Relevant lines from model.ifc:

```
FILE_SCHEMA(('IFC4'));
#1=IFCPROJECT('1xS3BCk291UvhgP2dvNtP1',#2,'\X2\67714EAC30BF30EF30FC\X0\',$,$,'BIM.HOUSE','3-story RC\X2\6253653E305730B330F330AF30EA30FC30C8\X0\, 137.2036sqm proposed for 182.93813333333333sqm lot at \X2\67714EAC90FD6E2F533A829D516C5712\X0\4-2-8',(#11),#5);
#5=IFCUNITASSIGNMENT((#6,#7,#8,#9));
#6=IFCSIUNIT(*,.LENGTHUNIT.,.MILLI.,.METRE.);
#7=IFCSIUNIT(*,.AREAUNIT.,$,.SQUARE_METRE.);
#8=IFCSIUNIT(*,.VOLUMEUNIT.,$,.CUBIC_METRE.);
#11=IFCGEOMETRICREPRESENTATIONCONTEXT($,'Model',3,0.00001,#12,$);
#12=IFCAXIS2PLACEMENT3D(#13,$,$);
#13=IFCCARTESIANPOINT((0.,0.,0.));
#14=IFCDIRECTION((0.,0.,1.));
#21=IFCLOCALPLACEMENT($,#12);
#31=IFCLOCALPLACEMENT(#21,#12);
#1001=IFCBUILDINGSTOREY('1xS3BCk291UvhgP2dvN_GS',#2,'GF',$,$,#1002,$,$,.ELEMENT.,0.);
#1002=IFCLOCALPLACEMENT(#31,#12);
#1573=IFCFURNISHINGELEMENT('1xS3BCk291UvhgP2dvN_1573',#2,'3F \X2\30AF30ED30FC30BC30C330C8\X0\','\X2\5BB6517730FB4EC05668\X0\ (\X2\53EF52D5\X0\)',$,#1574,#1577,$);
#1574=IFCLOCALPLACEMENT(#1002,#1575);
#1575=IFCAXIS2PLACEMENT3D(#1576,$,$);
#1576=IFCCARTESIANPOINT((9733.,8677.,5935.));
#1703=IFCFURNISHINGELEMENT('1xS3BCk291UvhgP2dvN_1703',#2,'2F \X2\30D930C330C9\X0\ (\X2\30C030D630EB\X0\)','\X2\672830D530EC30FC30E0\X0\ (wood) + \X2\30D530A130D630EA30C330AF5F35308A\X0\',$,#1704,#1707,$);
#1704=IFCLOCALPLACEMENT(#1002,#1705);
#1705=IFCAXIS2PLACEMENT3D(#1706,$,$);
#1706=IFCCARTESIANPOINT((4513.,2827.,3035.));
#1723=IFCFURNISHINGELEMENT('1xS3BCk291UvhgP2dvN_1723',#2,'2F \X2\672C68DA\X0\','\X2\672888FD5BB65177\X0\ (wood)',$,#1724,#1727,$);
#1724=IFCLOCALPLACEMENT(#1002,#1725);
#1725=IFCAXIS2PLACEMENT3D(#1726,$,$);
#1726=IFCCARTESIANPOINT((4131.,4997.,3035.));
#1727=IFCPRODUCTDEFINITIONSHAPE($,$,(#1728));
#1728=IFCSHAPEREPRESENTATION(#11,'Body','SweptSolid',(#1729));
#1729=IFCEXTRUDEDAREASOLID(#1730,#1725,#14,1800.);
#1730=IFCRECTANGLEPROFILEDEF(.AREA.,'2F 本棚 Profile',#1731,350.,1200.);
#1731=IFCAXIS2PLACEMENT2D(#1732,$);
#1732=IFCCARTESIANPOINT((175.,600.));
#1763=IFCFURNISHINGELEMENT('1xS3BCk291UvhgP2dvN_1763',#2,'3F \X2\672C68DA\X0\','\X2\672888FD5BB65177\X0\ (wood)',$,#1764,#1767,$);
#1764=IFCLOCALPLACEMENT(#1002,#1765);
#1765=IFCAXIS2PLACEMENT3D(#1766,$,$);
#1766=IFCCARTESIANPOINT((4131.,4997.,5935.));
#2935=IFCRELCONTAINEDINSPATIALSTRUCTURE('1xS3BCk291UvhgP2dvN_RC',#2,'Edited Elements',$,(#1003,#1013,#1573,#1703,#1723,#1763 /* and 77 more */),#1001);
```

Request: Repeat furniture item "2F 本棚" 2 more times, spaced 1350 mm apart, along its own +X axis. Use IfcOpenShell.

```python
import ifcopenshell
import ifcopenshell.api.geometry
import ifcopenshell.api.root
import ifcopenshell.util.element
import ifcopenshell.util.placement
import ifcopenshell.util.unit

model = ifcopenshell.open("model.ifc")
unit_scale = ifcopenshell.util.unit.calculate_unit_scale(model)


def reuse_history(source, copy):
    """copy_class also copies each property set's owner history, people and application; keep the originals."""
    for rel in copy.IsDefinedBy:
        if rel.is_a("IfcRelDefinesByProperties") and (history := rel.RelatingPropertyDefinition.OwnerHistory):
            rel.RelatingPropertyDefinition.OwnerHistory = source.OwnerHistory
            ifcopenshell.util.element.remove_deep2(model, history)


source = model.by_id(1723)
base = ifcopenshell.util.placement.get_local_placement(source.ObjectPlacement)
step = base[:3, 0] * 1.35 / unit_scale

for i in range(1, 3):
    copy = ifcopenshell.api.root.copy_class(model, product=source)
    copy.Representation = ifcopenshell.util.element.copy_deep(
        model, source.Representation, exclude=["IfcGeometricRepresentationContext", "IfcRepresentationMap"]
    )
    reuse_history(source, copy)
    matrix = base.copy()
    matrix[:3, 3] += i * step
    print("added at", matrix[:3, 3].round(3) + 0.0)
    ifcopenshell.api.geometry.edit_object_placement(model, product=copy, matrix=matrix, is_si=False)

model.write("model-out.ifc")
```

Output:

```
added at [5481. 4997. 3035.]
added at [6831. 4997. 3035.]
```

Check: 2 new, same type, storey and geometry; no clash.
